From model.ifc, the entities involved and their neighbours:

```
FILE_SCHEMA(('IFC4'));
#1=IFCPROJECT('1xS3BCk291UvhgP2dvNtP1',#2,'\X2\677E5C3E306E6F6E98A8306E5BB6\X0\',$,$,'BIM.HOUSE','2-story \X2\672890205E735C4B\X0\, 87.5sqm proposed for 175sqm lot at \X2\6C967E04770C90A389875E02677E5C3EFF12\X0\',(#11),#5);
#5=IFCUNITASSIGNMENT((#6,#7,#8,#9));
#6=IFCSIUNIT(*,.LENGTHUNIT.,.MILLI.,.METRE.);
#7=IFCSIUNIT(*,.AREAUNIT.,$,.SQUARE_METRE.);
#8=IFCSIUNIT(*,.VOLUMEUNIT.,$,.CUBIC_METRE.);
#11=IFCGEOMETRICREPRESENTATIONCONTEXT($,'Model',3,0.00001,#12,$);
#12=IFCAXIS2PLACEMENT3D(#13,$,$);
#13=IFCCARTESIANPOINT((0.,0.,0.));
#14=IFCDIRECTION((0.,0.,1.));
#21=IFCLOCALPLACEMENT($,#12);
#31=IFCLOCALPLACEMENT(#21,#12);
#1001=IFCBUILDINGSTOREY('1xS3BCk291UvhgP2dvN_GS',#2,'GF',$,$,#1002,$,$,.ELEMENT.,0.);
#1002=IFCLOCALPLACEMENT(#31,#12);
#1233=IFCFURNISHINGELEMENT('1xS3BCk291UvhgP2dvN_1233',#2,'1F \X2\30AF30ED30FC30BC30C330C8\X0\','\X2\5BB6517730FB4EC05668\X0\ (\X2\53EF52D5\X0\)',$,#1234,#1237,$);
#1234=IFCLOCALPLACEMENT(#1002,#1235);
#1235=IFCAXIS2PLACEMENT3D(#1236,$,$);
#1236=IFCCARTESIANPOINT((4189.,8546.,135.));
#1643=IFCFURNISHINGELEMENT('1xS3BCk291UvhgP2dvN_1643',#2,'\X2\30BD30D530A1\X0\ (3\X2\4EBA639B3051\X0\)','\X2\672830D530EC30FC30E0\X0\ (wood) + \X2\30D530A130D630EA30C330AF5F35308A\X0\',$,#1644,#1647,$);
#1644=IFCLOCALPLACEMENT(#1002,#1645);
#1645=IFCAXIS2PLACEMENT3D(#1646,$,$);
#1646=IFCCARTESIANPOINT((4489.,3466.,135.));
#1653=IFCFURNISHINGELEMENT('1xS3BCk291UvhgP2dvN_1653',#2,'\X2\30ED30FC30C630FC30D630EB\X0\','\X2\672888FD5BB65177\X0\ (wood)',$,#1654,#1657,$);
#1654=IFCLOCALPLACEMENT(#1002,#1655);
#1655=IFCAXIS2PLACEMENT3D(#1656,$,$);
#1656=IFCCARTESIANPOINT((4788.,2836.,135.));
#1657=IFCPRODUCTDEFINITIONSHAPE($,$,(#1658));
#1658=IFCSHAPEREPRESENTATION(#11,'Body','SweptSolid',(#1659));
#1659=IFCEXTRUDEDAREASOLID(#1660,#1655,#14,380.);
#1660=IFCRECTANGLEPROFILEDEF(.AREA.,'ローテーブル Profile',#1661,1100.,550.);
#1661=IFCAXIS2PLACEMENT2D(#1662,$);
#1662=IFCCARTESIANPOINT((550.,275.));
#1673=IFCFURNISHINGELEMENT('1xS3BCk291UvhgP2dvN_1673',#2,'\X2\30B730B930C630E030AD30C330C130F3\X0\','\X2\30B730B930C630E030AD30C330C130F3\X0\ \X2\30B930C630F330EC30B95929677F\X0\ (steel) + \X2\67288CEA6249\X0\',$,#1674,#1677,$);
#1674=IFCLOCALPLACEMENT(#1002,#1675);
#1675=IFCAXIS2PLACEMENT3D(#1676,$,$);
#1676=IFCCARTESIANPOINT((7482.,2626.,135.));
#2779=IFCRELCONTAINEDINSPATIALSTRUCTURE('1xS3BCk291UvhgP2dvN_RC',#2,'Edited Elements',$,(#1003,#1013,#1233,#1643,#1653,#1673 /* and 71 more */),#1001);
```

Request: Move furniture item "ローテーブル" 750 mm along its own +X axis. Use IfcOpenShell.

```python
import ifcopenshell
import ifcopenshell.api.geometry
import ifcopenshell.util.placement
import ifcopenshell.util.unit

model = ifcopenshell.open("model.ifc")
unit_scale = ifcopenshell.util.unit.calculate_unit_scale(model)

item = model.by_id(1653)
matrix = ifcopenshell.util.placement.get_local_placement(item.ObjectPlacement)
matrix[:3, 3] += matrix[:3, 0] * 0.75 / unit_scale
ifcopenshell.api.geometry.edit_object_placement(model, product=item, matrix=matrix, is_si=False)

print(ifcopenshell.util.placement.get_local_placement(item.ObjectPlacement).round(3) + 0.0)

model.write("model-out.ifc")
```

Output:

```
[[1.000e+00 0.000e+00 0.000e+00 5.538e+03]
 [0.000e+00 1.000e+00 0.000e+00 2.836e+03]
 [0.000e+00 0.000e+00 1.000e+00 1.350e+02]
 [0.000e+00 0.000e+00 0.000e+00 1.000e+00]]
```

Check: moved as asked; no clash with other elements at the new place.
